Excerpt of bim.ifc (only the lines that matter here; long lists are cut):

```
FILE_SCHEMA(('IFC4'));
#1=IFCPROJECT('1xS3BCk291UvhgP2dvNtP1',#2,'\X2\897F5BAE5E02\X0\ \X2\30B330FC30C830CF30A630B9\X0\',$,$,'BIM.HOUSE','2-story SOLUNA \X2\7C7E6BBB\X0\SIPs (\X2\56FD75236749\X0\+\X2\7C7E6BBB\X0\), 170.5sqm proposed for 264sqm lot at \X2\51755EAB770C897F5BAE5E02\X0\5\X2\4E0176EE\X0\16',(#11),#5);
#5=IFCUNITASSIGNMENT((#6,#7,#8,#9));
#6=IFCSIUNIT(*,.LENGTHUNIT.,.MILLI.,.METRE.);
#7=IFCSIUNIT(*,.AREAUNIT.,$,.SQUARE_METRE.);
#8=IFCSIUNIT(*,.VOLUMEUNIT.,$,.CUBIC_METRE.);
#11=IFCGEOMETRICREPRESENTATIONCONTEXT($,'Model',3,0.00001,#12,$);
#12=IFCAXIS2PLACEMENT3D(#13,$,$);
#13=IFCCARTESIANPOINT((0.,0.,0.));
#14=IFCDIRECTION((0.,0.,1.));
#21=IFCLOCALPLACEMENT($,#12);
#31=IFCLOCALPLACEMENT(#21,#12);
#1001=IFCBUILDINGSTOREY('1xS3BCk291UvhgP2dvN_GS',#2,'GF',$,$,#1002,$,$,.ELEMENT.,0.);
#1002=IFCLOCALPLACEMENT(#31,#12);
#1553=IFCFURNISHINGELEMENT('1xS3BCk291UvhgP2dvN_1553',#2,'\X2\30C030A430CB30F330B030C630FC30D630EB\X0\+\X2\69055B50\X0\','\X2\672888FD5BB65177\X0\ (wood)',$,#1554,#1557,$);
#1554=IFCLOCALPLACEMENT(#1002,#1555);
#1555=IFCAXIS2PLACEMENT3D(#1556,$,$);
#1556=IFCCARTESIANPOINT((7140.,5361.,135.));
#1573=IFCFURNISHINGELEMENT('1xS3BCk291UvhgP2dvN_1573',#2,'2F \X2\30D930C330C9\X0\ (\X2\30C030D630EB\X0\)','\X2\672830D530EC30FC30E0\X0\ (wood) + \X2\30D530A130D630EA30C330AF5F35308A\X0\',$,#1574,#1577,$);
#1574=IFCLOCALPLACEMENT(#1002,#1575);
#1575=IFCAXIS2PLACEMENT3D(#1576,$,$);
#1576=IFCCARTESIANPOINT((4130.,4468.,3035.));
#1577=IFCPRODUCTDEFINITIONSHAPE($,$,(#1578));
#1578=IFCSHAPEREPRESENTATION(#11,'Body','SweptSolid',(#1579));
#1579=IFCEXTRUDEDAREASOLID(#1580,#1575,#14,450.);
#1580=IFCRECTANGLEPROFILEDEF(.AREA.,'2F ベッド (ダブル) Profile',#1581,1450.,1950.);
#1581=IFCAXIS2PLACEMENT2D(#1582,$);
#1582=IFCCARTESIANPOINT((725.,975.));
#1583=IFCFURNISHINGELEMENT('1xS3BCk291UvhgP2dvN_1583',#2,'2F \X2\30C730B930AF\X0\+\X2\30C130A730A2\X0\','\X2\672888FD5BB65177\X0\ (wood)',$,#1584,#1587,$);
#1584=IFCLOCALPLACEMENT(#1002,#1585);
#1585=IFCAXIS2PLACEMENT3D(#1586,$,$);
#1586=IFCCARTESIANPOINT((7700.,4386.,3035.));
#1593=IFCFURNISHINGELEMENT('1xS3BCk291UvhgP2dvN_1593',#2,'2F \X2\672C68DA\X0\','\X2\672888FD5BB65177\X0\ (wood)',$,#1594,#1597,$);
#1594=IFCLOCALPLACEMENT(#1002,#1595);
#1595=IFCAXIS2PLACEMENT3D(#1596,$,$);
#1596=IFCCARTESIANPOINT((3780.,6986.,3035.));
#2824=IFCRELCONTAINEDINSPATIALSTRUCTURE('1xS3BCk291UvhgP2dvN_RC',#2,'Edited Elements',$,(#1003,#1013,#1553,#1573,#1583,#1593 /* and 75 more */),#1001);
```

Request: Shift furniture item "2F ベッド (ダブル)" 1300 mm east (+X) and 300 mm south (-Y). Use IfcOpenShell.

```python
import ifcopenshell
import ifcopenshell.api.geometry
import ifcopenshell.util.placement
import ifcopenshell.util.unit

model = ifcopenshell.open("bim.ifc")
unit_scale = ifcopenshell.util.unit.calculate_unit_scale(model)

item = model.by_guid("1xS3BCk291UvhgP2dvN_1573")
matrix = ifcopenshell.util.placement.get_local_placement(item.ObjectPlacement)
matrix[0, 3] += 1.3 / unit_scale
matrix[1, 3] -= 0.3 / unit_scale
ifcopenshell.api.geometry.edit_object_placement(model, product=item, matrix=matrix, is_si=False)

print(ifcopenshell.util.placement.get_local_placement(item.ObjectPlacement).round(3) + 0.0)

model.write("bim-out.ifc")
```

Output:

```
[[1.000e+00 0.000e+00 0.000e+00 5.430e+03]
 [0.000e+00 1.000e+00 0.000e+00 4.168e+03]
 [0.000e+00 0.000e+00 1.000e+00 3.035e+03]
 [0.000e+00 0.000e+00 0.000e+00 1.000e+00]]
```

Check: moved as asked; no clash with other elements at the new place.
